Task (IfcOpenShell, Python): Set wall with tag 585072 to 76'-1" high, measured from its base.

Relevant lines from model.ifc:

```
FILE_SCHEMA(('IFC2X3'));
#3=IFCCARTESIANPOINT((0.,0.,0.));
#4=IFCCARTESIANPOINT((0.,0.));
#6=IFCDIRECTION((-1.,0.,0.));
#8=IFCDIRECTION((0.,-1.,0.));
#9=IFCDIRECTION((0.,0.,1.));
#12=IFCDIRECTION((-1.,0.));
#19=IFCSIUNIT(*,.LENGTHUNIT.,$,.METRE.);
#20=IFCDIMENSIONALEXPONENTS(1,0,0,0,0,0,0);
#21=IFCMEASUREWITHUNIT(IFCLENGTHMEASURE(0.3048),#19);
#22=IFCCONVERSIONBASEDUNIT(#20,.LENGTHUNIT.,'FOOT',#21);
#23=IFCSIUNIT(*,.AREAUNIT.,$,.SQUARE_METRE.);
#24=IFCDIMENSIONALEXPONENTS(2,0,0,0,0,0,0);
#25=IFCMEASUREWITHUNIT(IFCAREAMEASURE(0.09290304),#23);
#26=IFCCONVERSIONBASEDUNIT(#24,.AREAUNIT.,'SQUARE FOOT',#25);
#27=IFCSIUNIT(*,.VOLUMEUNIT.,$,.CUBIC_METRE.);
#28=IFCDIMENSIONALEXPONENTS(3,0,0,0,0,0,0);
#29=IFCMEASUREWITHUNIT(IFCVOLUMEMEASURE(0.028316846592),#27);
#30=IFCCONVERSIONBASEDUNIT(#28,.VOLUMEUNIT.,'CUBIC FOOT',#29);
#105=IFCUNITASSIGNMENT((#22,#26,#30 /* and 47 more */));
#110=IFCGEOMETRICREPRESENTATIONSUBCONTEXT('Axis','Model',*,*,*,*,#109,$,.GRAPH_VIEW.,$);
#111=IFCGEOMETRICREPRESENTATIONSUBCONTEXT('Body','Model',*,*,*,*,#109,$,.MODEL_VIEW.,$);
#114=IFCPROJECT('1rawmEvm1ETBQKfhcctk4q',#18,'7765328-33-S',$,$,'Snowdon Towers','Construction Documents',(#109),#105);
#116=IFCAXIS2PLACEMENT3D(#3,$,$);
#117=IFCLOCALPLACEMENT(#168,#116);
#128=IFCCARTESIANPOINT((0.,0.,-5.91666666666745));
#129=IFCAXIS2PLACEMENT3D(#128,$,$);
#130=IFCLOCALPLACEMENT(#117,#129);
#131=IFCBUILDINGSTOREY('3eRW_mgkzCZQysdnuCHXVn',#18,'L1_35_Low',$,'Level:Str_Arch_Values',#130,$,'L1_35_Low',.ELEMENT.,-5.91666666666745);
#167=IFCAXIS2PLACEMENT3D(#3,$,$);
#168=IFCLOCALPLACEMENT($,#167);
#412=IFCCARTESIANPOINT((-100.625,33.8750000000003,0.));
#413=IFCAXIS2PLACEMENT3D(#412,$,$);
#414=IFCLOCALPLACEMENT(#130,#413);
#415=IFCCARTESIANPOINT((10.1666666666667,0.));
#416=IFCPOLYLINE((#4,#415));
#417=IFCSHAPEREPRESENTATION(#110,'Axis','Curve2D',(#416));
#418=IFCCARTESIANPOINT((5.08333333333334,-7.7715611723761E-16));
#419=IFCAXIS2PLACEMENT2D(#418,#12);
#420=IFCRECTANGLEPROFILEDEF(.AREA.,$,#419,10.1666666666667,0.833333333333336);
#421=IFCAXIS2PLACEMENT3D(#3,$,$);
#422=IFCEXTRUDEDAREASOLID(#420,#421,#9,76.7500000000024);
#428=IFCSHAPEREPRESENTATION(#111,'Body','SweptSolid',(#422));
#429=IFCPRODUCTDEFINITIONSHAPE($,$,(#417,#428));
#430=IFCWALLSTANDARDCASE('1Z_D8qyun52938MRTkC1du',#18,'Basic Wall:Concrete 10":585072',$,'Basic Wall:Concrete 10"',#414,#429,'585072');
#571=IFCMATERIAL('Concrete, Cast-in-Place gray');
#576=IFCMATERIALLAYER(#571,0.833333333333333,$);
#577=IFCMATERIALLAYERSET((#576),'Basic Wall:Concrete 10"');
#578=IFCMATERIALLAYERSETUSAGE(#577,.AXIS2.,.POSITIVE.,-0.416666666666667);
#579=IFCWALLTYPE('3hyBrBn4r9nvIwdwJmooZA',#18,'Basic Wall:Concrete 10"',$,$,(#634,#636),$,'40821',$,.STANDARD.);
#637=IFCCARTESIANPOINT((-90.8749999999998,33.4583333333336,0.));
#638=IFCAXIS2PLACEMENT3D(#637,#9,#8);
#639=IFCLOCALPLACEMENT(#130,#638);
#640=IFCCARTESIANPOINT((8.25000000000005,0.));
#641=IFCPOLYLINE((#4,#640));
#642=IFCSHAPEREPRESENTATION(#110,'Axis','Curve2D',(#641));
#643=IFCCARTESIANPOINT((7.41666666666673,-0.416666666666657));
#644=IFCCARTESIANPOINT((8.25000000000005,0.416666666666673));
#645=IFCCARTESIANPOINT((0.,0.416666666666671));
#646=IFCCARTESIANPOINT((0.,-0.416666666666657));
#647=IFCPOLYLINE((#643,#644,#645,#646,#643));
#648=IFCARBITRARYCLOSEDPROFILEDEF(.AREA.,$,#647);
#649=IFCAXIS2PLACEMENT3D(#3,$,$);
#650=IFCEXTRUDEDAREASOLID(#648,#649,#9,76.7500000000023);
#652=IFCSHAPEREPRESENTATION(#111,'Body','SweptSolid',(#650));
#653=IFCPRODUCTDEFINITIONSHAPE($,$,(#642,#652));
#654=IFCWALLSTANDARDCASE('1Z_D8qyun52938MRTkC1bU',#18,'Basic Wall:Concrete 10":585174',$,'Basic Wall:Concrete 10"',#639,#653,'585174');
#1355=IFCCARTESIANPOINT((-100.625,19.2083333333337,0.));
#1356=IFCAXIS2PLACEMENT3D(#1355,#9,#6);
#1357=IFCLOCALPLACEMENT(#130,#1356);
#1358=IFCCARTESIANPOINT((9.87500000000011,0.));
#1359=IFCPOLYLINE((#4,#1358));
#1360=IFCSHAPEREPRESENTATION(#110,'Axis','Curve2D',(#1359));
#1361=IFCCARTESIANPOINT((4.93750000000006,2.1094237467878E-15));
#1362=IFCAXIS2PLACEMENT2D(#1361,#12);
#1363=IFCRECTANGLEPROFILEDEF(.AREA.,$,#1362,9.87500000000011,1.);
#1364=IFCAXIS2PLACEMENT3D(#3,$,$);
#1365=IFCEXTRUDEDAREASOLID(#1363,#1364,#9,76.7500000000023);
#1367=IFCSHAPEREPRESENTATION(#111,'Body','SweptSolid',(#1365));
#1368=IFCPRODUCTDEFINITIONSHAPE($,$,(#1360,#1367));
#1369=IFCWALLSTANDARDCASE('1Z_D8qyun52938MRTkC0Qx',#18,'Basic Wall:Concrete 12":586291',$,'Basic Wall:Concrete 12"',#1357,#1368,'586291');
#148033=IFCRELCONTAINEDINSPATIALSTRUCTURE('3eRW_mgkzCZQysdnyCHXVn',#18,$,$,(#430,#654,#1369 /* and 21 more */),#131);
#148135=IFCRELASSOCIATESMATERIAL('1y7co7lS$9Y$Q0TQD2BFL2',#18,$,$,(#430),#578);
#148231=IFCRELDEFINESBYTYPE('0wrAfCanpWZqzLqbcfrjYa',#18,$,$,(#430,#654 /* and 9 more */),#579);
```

```python
import ifcopenshell
import ifcopenshell.geom
import ifcopenshell.util.representation
import ifcopenshell.util.shape
import ifcopenshell.util.unit

model = ifcopenshell.open("model.ifc")
unit_scale = ifcopenshell.util.unit.calculate_unit_scale(model)
settings = ifcopenshell.geom.settings()


def volume(element):
    """Net volume in cubic metres, openings subtracted."""
    shape = ifcopenshell.geom.create_shape(settings, element)
    return ifcopenshell.util.shape.get_volume(shape.geometry)


wall = model.by_id(430)
before = volume(wall)

body = ifcopenshell.util.representation.get_representation(wall, "Model", "Body")
solid = body.Items[0]
old_height = solid.Depth
solid.Depth = 913 * 0.0254 / unit_scale
after = volume(wall)

print(f"height {old_height:g} -> {solid.Depth:g}, volume {before:.3f} -> {after:.3f} m3")

model.write("model_updated.ifc")
```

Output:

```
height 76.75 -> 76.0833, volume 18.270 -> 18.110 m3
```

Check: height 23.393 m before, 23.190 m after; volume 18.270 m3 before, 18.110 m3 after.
